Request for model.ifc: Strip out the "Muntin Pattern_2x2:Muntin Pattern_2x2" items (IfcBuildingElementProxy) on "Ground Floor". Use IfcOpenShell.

First a look at what the model holds.

```python
import ifcopenshell
import ifcopenshell.util.element

model = ifcopenshell.open("model.ifc")
print(model.schema)
storey = next(s for s in model.by_type("IfcBuildingStorey") if s.Name == "Ground Floor")
proxies = [e for e in ifcopenshell.util.element.get_decomposition(storey) if e.is_a("IfcBuildingElementProxy")]
seen = {}
for e in proxies:
    element_type = ifcopenshell.util.element.get_type(e)
    name = element_type.Name if element_type not in (None, e) else None
    seen[name] = seen.get(name, 0) + 1
for name, count in sorted(seen.items(), key=str):
    print(count, "x", name)
```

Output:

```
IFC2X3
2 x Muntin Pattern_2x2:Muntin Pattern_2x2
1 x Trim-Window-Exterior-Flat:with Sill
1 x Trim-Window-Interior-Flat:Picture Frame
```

```python
import ifcopenshell
import ifcopenshell.api.root
import ifcopenshell.util.element

model = ifcopenshell.open("model.ifc")

storey = next(s for s in model.by_type("IfcBuildingStorey") if s.Name == "Ground Floor")
proxies = [e for e in ifcopenshell.util.element.get_decomposition(storey) if e.is_a("IfcBuildingElementProxy")]
targets = [e for e in proxies if (t := ifcopenshell.util.element.get_type(e)) not in (None, e) and t.Name == "Muntin Pattern_2x2:Muntin Pattern_2x2"]

for e in targets:
    ifcopenshell.api.root.remove_product(model, product=e)
print(len(targets), "removed")

model.write("model_rev.ifc")
```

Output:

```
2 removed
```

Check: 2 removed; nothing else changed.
